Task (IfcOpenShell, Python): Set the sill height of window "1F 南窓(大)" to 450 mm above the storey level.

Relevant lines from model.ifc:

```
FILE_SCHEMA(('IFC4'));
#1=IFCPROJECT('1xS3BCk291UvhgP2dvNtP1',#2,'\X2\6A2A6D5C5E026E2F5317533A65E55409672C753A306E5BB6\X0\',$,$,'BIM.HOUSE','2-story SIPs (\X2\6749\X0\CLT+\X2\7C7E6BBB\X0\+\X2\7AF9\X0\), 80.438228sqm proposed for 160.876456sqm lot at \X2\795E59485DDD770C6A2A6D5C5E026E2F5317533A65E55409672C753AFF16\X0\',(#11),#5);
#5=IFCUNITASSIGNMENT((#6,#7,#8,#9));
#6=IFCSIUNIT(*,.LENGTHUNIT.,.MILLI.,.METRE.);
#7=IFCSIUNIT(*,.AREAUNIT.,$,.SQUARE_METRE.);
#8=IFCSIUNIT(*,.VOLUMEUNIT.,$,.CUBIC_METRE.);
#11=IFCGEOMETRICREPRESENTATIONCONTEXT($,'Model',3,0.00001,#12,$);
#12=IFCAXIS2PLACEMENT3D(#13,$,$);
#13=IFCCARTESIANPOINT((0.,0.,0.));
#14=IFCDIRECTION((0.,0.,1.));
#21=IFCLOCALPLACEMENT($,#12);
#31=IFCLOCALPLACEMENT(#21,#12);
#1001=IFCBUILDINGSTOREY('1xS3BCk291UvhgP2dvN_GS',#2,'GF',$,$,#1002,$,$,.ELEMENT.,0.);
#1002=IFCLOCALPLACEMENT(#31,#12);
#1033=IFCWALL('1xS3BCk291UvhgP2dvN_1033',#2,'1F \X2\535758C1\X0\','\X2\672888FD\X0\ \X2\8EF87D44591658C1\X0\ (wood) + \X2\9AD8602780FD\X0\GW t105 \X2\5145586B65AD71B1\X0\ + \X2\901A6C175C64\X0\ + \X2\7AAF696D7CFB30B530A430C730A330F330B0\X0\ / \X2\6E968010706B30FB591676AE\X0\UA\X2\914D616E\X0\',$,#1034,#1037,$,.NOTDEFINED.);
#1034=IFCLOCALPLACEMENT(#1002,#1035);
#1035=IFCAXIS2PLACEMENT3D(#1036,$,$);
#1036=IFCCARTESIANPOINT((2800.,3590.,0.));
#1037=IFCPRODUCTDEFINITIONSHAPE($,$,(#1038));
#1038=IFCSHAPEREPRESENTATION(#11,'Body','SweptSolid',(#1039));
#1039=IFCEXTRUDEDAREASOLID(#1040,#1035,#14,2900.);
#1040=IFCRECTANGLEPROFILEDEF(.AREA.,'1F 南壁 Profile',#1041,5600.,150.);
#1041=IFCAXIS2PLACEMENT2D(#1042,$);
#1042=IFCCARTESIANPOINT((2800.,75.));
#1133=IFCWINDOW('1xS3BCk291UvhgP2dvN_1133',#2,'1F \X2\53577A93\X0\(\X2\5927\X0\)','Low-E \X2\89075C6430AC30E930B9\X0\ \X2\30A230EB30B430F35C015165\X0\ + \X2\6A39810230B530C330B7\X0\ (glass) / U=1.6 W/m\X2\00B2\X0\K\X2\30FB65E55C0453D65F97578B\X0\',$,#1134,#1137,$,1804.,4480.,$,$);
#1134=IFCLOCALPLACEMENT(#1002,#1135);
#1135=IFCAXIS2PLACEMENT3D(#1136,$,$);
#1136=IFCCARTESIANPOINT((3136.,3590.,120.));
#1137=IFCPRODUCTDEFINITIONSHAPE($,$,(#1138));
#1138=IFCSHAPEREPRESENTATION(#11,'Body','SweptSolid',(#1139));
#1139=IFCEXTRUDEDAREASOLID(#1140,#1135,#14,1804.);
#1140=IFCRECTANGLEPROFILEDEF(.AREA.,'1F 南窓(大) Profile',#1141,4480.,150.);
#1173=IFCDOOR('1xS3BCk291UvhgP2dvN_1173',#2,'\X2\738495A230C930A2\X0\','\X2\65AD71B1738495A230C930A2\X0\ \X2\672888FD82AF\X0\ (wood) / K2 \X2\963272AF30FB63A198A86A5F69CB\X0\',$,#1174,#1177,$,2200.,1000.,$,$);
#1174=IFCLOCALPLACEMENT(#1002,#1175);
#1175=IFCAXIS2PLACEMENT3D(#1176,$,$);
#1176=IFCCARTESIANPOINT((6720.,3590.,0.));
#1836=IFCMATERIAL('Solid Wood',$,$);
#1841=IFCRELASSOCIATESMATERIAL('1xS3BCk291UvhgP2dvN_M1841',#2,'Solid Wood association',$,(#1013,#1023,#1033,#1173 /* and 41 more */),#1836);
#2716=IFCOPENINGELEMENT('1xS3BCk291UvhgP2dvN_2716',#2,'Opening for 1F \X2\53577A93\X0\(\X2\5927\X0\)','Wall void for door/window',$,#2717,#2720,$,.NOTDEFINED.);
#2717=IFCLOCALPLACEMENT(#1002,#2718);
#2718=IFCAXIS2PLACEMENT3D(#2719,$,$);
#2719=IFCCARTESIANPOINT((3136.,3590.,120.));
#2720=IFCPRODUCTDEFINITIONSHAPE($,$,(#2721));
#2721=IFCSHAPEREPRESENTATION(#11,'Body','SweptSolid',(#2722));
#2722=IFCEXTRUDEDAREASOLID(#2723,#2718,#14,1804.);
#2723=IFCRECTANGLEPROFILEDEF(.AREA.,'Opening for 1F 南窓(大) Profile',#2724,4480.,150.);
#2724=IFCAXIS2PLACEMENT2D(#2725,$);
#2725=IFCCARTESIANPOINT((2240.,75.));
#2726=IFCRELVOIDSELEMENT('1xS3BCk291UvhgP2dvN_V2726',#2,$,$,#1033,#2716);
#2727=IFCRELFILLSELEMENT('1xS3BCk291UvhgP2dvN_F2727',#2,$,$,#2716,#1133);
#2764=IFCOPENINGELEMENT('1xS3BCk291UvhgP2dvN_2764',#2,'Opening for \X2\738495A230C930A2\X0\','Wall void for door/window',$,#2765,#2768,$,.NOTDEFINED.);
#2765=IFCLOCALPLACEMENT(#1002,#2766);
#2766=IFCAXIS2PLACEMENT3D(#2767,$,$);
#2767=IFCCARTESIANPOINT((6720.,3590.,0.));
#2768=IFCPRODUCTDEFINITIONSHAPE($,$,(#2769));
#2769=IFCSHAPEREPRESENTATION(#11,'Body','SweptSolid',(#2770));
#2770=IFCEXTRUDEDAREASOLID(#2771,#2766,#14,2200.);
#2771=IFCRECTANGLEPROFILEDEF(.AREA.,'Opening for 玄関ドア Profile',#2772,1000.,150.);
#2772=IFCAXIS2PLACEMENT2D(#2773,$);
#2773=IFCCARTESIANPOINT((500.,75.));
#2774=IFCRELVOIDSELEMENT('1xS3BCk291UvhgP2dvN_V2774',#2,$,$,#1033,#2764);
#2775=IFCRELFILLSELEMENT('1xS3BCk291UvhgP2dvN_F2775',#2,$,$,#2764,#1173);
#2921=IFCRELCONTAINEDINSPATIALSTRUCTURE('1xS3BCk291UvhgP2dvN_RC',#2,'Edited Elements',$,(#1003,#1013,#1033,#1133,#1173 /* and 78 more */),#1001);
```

```python
import numpy as np
import ifcopenshell
import ifcopenshell.api.geometry
import ifcopenshell.geom
import ifcopenshell.util.element
import ifcopenshell.util.placement
import ifcopenshell.util.shape
import ifcopenshell.util.unit

model = ifcopenshell.open("model.ifc")
unit_scale = ifcopenshell.util.unit.calculate_unit_scale(model)

window = model.by_guid("1xS3BCk291UvhgP2dvN_1133")
opening = window.FillsVoids[0].RelatingOpeningElement
storey = ifcopenshell.util.element.get_container(window, ifc_class="IfcBuildingStorey")
level = ifcopenshell.util.placement.get_local_placement(storey.ObjectPlacement)[2, 3]

# The opening's origin need not be at the sill, so measure its lowest point.
shape = ifcopenshell.geom.create_shape(ifcopenshell.geom.settings(), opening)
bottom = ifcopenshell.util.shape.get_shape_bottom_elevation(shape, shape.geometry) / unit_scale
dz = level + 0.45 / unit_scale - bottom

shift = np.array([0.0, 0.0, dz])
# The window is not placed relative to its opening, so move both.
for product in (opening, window):
    matrix = ifcopenshell.util.placement.get_local_placement(product.ObjectPlacement)
    matrix[:3, 3] += shift
    ifcopenshell.api.geometry.edit_object_placement(model, product=product, matrix=matrix, is_si=False)

print(f"moved by {dz * unit_scale:+.3f} m")

model.write("model_v2.ifc")
```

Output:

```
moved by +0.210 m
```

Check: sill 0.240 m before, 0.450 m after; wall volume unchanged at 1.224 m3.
